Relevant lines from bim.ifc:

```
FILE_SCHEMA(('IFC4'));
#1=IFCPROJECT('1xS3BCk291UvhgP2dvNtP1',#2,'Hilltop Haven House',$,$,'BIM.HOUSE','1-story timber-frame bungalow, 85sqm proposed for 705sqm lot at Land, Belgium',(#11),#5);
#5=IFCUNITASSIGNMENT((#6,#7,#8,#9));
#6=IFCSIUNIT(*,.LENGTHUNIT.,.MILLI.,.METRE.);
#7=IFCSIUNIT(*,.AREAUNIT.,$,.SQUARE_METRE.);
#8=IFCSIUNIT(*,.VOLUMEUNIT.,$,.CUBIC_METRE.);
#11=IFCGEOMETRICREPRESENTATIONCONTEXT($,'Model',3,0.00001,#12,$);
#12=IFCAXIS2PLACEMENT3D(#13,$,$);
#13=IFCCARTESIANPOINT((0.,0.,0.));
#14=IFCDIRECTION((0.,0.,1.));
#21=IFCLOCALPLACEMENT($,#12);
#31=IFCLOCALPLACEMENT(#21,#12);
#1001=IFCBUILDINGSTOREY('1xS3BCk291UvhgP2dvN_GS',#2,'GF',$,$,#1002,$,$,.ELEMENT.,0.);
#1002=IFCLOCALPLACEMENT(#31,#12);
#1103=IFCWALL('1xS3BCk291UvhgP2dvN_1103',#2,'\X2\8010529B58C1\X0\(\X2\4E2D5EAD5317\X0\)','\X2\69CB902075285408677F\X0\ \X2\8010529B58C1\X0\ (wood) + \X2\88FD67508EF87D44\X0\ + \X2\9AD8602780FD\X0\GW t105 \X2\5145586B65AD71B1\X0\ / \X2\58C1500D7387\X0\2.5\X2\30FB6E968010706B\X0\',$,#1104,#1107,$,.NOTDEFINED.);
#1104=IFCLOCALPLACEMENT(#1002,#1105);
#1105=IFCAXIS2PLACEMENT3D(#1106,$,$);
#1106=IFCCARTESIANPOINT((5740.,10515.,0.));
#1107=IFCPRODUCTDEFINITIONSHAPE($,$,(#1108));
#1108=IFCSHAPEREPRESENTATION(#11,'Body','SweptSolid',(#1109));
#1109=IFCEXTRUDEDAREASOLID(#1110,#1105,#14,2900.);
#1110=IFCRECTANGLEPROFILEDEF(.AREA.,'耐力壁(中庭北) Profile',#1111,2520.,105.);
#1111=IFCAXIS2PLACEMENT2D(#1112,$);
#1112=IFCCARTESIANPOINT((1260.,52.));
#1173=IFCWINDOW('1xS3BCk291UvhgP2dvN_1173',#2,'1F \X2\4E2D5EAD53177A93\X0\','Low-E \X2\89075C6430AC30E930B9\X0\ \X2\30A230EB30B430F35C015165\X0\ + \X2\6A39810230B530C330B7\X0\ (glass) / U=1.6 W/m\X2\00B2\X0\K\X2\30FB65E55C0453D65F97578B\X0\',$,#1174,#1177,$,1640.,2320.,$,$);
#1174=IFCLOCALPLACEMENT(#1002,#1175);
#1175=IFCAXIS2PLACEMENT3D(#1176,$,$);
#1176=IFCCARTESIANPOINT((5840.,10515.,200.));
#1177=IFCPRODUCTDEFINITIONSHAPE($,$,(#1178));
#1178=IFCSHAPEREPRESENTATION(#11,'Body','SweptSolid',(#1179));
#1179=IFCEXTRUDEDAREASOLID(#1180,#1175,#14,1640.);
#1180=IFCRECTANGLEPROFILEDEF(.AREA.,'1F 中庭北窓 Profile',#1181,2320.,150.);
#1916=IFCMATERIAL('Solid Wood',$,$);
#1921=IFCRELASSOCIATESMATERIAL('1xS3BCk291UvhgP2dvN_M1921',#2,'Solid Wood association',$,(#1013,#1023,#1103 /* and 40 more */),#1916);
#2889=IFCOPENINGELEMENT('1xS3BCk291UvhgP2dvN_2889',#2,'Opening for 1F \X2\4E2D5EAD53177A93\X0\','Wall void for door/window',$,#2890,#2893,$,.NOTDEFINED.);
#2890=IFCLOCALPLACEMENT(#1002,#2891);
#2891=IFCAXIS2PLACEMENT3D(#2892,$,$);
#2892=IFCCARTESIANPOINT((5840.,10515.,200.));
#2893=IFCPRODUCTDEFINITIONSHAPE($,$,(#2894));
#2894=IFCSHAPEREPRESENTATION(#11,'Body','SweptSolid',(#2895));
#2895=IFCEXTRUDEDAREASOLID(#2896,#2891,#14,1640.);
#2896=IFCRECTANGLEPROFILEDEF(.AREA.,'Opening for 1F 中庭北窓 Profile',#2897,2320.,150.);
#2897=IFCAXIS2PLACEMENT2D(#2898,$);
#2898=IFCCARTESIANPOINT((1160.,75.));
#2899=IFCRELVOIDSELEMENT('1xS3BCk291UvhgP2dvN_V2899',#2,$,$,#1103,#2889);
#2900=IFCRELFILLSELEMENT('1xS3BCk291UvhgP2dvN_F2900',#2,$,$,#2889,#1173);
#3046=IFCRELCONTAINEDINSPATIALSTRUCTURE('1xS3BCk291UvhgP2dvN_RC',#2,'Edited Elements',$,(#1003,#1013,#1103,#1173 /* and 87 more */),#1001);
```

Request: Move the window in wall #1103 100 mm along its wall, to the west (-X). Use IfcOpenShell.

```python
import ifcopenshell
import ifcopenshell.api.geometry
import ifcopenshell.util.placement
import ifcopenshell.util.unit

model = ifcopenshell.open("bim.ifc")
unit_scale = ifcopenshell.util.unit.calculate_unit_scale(model)

window = model.by_guid("1xS3BCk291UvhgP2dvN_1173")
opening = window.FillsVoids[0].RelatingOpeningElement
wall = opening.VoidsElements[0].RelatingBuildingElement

wall_matrix = ifcopenshell.util.placement.get_local_placement(wall.ObjectPlacement)
shift = wall_matrix[:3, 0] * -0.1 / unit_scale
before = ifcopenshell.util.placement.get_local_placement(window.ObjectPlacement)[:3, 3].copy()

# The window is not placed relative to its opening, so move both.
for product in (opening, window):
    matrix = ifcopenshell.util.placement.get_local_placement(product.ObjectPlacement)
    matrix[:3, 3] += shift
    ifcopenshell.api.geometry.edit_object_placement(model, product=product, matrix=matrix, is_si=False)

after = ifcopenshell.util.placement.get_local_placement(window.ObjectPlacement)[:3, 3]
print("window moved by", (after - before).round(3) + 0.0)

model.write("bim_rev.ifc")
```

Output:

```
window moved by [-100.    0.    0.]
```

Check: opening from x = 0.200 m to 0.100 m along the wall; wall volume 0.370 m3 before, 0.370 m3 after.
